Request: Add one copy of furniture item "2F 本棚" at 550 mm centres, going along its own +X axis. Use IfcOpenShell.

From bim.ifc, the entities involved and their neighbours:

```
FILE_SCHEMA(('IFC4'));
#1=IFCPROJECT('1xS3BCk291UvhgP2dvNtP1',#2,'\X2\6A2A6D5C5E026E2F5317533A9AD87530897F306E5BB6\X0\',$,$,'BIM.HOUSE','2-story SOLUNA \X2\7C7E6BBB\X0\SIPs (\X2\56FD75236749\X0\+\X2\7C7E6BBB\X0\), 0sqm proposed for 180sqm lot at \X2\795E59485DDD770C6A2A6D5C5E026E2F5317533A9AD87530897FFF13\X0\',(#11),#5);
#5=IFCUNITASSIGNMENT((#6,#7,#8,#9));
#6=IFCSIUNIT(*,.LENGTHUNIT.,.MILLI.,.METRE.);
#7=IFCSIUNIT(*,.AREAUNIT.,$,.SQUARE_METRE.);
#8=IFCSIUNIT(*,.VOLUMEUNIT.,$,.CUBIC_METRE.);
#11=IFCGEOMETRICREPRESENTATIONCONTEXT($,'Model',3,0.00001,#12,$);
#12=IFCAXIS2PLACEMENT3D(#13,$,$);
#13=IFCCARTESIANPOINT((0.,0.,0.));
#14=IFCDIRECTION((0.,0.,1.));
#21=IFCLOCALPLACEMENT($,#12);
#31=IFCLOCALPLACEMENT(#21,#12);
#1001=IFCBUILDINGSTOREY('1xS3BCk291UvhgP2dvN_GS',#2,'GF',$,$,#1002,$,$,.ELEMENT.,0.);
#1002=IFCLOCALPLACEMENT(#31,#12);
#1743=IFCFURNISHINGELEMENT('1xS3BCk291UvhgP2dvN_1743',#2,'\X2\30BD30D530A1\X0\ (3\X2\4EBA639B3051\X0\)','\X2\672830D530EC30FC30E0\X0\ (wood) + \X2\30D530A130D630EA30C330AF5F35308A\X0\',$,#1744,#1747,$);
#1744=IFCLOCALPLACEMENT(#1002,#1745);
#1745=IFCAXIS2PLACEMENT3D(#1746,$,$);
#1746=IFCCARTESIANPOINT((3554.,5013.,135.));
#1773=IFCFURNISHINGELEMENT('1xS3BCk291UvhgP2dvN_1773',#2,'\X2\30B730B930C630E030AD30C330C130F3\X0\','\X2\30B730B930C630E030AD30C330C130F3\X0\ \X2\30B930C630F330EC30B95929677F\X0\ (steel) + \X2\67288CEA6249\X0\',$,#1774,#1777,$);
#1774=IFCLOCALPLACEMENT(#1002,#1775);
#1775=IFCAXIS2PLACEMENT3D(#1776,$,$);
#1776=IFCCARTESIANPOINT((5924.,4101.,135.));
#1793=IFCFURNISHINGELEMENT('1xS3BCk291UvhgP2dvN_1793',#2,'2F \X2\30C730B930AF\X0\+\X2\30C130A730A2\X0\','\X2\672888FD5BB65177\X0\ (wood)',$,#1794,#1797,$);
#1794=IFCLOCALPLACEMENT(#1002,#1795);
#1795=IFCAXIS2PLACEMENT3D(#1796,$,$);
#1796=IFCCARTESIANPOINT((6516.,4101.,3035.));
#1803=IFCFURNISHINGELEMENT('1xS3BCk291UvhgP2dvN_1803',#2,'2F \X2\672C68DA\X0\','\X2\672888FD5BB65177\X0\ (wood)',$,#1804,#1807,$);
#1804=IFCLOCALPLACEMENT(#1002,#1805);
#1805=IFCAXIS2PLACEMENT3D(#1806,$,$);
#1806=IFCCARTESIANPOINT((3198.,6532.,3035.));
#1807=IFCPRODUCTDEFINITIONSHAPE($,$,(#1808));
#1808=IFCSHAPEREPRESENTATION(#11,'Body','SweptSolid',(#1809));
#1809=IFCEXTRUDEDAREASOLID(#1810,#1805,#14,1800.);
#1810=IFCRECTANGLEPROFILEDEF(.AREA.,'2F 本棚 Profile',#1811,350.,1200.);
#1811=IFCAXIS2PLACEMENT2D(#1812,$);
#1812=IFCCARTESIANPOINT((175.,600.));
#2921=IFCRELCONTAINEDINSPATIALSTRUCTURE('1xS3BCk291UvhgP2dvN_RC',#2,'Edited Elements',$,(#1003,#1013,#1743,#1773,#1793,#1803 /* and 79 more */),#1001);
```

```python
import ifcopenshell
import ifcopenshell.api.geometry
import ifcopenshell.api.root
import ifcopenshell.util.element
import ifcopenshell.util.placement
import ifcopenshell.util.unit

model = ifcopenshell.open("bim.ifc")
unit_scale = ifcopenshell.util.unit.calculate_unit_scale(model)


def reuse_history(source, copy):
    """copy_class also copies each property set's owner history, people and application; keep the originals."""
    for rel in copy.IsDefinedBy:
        if rel.is_a("IfcRelDefinesByProperties") and (history := rel.RelatingPropertyDefinition.OwnerHistory):
            rel.RelatingPropertyDefinition.OwnerHistory = source.OwnerHistory
            ifcopenshell.util.element.remove_deep2(model, history)


source = model.by_guid("1xS3BCk291UvhgP2dvN_1803")
base = ifcopenshell.util.placement.get_local_placement(source.ObjectPlacement)
step = base[:3, 0] * 0.55 / unit_scale

for i in range(1, 2):
    copy = ifcopenshell.api.root.copy_class(model, product=source)
    copy.Representation = ifcopenshell.util.element.copy_deep(
        model, source.Representation, exclude=["IfcGeometricRepresentationContext", "IfcRepresentationMap"]
    )
    reuse_history(source, copy)
    matrix = base.copy()
    matrix[:3, 3] += i * step
    print("added at", matrix[:3, 3].round(3) + 0.0)
    ifcopenshell.api.geometry.edit_object_placement(model, product=copy, matrix=matrix, is_si=False)

model.write("bim_updated.ifc")
```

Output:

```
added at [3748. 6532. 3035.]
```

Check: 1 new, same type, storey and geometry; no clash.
